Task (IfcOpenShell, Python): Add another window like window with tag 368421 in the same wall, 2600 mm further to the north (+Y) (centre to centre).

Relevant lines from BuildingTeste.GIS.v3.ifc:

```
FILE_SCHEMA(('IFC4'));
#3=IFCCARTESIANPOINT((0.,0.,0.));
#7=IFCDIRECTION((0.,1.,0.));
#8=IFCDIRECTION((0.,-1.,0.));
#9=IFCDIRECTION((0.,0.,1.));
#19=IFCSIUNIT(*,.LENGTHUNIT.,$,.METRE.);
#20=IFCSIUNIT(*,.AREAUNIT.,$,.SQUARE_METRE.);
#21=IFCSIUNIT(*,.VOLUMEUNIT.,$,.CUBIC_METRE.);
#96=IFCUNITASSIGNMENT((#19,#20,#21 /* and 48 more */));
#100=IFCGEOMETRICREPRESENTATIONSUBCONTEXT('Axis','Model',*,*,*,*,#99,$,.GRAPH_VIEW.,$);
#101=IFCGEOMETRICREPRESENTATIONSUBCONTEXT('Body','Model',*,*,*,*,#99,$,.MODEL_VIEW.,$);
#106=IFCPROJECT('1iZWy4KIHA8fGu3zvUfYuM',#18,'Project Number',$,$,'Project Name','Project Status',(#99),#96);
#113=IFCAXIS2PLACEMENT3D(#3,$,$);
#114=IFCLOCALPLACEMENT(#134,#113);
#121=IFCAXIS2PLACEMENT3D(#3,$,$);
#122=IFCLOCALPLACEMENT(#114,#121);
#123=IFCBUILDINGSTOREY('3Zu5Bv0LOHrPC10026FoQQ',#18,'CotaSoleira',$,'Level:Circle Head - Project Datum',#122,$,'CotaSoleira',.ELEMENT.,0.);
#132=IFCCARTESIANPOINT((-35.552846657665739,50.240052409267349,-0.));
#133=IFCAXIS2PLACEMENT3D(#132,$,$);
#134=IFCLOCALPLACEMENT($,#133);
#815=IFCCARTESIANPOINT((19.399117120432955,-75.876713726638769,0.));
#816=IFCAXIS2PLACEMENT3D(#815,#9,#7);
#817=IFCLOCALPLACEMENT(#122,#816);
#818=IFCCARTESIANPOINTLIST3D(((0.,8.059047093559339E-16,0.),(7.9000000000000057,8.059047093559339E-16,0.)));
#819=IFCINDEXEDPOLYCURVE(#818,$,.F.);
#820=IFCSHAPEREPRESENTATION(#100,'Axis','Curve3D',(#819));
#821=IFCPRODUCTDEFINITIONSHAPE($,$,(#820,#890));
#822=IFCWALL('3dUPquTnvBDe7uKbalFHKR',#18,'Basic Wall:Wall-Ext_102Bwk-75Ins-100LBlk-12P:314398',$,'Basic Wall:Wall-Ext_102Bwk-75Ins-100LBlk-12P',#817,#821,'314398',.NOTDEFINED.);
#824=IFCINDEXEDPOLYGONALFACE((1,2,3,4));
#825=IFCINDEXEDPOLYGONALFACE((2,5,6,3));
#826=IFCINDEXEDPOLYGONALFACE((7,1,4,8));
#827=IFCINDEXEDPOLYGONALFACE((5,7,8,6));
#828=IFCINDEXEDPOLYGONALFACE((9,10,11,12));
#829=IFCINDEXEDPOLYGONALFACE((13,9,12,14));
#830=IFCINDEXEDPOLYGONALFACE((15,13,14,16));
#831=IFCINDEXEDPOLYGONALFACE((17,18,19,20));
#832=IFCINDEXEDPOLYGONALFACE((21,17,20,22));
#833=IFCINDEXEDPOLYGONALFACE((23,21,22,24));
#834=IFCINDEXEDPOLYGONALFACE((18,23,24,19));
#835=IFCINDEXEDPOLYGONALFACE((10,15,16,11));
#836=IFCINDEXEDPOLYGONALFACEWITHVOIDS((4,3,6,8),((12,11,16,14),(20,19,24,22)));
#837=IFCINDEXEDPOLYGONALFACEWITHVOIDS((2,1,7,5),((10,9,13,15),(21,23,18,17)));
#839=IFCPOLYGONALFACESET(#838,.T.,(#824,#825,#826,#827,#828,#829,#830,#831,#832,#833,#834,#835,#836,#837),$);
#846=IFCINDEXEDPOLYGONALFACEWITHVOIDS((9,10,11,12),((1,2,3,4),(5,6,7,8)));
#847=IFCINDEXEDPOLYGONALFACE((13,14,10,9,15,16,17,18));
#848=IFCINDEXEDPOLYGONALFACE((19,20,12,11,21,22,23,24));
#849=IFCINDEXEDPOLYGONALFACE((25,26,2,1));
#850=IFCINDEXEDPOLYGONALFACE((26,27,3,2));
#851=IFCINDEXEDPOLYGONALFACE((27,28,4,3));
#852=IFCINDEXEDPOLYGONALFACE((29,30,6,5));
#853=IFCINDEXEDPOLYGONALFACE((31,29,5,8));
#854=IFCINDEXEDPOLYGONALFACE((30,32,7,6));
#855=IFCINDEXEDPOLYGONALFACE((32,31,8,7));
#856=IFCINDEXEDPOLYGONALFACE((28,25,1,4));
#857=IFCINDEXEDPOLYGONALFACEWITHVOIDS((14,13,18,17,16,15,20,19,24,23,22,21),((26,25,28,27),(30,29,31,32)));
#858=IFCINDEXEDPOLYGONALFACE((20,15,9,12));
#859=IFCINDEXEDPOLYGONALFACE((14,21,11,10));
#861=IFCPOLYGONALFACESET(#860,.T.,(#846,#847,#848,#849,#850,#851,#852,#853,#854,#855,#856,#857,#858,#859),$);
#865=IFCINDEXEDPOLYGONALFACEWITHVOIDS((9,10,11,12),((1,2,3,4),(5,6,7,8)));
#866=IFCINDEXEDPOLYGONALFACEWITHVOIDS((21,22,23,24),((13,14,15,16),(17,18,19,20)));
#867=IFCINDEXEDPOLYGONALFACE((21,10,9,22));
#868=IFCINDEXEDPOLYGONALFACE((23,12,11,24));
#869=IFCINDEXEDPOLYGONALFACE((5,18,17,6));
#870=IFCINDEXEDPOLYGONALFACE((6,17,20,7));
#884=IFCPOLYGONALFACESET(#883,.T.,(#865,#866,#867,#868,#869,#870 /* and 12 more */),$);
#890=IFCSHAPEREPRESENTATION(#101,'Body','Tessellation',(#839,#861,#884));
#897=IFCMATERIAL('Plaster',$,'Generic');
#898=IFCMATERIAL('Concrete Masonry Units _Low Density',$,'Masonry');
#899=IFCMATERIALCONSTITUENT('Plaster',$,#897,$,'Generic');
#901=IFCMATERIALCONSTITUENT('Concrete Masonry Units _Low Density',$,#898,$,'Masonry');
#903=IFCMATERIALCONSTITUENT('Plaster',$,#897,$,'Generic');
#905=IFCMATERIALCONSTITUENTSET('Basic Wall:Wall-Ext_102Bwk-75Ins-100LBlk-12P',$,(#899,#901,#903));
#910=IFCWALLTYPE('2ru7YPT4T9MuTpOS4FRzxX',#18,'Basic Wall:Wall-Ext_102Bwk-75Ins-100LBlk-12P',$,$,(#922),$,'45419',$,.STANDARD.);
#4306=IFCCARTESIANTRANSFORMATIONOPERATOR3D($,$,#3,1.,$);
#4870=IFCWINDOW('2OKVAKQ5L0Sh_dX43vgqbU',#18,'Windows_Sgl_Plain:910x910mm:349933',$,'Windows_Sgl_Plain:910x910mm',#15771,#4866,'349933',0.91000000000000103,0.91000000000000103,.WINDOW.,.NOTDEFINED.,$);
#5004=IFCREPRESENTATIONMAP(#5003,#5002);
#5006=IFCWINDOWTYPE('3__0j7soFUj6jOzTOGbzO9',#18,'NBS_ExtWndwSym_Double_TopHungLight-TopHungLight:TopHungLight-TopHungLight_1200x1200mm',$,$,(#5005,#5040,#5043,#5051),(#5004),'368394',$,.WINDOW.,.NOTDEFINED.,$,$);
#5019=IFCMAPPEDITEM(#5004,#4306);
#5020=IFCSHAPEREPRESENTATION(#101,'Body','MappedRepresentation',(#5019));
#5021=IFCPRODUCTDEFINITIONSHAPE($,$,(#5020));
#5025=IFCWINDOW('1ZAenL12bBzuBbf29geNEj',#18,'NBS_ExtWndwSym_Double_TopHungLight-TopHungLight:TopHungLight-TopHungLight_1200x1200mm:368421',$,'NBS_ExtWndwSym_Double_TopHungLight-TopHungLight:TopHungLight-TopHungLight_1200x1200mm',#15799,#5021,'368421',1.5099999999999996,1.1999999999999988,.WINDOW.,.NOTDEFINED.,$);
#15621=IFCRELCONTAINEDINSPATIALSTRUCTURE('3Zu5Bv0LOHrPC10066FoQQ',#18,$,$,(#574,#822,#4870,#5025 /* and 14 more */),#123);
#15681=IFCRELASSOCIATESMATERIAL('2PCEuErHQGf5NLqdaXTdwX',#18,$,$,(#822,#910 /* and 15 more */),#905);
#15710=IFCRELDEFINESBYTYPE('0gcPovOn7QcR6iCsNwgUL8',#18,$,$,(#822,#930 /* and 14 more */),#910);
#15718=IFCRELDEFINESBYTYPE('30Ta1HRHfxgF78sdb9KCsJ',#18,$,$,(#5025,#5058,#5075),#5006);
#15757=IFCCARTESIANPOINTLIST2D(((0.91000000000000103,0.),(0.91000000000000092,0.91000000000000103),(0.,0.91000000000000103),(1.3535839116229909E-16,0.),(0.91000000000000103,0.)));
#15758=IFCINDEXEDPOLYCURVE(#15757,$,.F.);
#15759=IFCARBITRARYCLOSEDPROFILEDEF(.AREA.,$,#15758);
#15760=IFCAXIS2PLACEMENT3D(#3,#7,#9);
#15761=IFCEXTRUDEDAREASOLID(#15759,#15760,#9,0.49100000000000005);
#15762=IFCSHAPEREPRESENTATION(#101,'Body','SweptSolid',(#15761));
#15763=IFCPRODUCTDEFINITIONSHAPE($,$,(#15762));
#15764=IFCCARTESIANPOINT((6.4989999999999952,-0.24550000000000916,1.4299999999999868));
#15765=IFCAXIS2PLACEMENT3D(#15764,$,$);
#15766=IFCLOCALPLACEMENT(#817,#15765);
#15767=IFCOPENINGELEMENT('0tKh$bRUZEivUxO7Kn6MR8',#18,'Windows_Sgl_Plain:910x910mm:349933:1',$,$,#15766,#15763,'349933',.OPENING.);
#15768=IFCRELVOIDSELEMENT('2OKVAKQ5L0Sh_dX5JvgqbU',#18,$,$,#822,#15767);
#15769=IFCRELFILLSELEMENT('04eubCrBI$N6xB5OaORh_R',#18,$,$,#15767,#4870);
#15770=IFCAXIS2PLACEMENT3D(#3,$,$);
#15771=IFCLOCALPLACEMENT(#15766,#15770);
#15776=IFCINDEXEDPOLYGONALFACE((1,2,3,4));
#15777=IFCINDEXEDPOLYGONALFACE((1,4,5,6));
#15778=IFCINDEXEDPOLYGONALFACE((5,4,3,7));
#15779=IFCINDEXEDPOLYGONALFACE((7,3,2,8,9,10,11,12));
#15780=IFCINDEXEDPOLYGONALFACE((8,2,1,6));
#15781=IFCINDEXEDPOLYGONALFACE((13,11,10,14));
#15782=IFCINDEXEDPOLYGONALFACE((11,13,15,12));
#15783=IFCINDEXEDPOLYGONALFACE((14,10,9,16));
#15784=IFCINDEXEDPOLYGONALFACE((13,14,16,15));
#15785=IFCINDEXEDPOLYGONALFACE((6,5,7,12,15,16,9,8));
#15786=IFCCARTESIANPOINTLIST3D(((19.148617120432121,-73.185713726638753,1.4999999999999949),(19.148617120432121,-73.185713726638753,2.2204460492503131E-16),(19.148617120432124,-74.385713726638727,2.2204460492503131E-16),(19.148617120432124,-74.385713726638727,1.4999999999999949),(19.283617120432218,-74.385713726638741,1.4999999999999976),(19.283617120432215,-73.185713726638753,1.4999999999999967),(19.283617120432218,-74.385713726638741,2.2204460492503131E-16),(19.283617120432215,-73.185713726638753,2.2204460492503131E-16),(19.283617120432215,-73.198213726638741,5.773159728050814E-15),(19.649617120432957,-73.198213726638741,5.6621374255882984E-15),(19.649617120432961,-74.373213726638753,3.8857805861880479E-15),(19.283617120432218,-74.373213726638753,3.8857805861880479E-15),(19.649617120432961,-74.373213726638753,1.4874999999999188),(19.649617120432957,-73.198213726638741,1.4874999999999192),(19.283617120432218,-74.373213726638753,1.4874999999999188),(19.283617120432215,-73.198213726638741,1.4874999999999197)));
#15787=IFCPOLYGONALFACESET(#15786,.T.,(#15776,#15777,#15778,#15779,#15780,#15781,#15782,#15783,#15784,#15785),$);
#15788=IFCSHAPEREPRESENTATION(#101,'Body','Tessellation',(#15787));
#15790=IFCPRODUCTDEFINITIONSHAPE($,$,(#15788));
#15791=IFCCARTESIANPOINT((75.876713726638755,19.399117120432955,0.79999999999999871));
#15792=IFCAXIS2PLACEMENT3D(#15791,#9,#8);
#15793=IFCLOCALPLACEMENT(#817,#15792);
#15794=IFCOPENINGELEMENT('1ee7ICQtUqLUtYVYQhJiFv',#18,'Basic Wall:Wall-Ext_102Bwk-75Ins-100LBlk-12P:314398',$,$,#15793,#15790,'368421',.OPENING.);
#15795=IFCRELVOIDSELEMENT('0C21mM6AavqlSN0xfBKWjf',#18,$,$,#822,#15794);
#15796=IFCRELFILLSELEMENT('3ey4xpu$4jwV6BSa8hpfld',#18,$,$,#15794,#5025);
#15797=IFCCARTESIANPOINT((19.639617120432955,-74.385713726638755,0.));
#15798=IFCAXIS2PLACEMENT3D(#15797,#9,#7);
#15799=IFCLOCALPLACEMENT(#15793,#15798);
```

```python
import ifcopenshell
import ifcopenshell.api.feature
import ifcopenshell.api.geometry
import ifcopenshell.api.root
import ifcopenshell.geom
import ifcopenshell.util.element
import ifcopenshell.util.placement
import ifcopenshell.util.shape
import ifcopenshell.util.unit

model = ifcopenshell.open("BuildingTeste.GIS.v3.ifc")
unit_scale = ifcopenshell.util.unit.calculate_unit_scale(model)
settings = ifcopenshell.geom.settings()


def volume(element):
    """Net volume in cubic metres, openings subtracted."""
    shape = ifcopenshell.geom.create_shape(settings, element)
    return ifcopenshell.util.shape.get_volume(shape.geometry)


def reuse_history(source, copy):
    """copy_class also copies each property set's owner history, people and application; keep the originals."""
    for rel in copy.IsDefinedBy:
        if rel.is_a("IfcRelDefinesByProperties") and (history := rel.RelatingPropertyDefinition.OwnerHistory):
            rel.RelatingPropertyDefinition.OwnerHistory = source.OwnerHistory
            ifcopenshell.util.element.remove_deep2(model, history)


window = model.by_id(5025)
opening = window.FillsVoids[0].RelatingOpeningElement
wall = opening.VoidsElements[0].RelatingBuildingElement
before = volume(wall)
shift = ifcopenshell.util.placement.get_local_placement(wall.ObjectPlacement)[:3, 0] * 2.6 / unit_scale

# copy_class copies the void relationship, type, container and properties, but no geometry.
new_opening = ifcopenshell.api.root.copy_class(model, product=opening)
new_opening.Representation = ifcopenshell.util.element.copy_deep(
    model, opening.Representation, exclude=["IfcGeometricRepresentationContext", "IfcRepresentationMap"]
)
new_opening.Name = "Basic Wall:Wall-Ext_102Bwk-75Ins-100LBlk-12P"
new_opening.Tag = None
new_window = ifcopenshell.api.root.copy_class(model, product=window)
new_window.Representation = ifcopenshell.util.element.copy_deep(
    model, window.Representation, exclude=["IfcGeometricRepresentationContext", "IfcRepresentationMap"]
)
new_window.Name = "NBS_ExtWndwSym_Double_TopHungLight-TopHungLight:TopHungLight-TopHungLight_1200x1200mm"
new_window.Tag = None
reuse_history(window, new_window)
ifcopenshell.api.feature.add_filling(model, opening=new_opening, element=new_window)

for old, new in ((opening, new_opening), (window, new_window)):
    matrix = ifcopenshell.util.placement.get_local_placement(old.ObjectPlacement)
    matrix[:3, 3] += shift
    ifcopenshell.api.geometry.edit_object_placement(model, product=new, matrix=matrix, is_si=False)

after = volume(wall)

print(f"wall volume {before:.3f} -> {after:.3f} m3")

model.write("BuildingTeste.GIS.v3-out.ifc")
```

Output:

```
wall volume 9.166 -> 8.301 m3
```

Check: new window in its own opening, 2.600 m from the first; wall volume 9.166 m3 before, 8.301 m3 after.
